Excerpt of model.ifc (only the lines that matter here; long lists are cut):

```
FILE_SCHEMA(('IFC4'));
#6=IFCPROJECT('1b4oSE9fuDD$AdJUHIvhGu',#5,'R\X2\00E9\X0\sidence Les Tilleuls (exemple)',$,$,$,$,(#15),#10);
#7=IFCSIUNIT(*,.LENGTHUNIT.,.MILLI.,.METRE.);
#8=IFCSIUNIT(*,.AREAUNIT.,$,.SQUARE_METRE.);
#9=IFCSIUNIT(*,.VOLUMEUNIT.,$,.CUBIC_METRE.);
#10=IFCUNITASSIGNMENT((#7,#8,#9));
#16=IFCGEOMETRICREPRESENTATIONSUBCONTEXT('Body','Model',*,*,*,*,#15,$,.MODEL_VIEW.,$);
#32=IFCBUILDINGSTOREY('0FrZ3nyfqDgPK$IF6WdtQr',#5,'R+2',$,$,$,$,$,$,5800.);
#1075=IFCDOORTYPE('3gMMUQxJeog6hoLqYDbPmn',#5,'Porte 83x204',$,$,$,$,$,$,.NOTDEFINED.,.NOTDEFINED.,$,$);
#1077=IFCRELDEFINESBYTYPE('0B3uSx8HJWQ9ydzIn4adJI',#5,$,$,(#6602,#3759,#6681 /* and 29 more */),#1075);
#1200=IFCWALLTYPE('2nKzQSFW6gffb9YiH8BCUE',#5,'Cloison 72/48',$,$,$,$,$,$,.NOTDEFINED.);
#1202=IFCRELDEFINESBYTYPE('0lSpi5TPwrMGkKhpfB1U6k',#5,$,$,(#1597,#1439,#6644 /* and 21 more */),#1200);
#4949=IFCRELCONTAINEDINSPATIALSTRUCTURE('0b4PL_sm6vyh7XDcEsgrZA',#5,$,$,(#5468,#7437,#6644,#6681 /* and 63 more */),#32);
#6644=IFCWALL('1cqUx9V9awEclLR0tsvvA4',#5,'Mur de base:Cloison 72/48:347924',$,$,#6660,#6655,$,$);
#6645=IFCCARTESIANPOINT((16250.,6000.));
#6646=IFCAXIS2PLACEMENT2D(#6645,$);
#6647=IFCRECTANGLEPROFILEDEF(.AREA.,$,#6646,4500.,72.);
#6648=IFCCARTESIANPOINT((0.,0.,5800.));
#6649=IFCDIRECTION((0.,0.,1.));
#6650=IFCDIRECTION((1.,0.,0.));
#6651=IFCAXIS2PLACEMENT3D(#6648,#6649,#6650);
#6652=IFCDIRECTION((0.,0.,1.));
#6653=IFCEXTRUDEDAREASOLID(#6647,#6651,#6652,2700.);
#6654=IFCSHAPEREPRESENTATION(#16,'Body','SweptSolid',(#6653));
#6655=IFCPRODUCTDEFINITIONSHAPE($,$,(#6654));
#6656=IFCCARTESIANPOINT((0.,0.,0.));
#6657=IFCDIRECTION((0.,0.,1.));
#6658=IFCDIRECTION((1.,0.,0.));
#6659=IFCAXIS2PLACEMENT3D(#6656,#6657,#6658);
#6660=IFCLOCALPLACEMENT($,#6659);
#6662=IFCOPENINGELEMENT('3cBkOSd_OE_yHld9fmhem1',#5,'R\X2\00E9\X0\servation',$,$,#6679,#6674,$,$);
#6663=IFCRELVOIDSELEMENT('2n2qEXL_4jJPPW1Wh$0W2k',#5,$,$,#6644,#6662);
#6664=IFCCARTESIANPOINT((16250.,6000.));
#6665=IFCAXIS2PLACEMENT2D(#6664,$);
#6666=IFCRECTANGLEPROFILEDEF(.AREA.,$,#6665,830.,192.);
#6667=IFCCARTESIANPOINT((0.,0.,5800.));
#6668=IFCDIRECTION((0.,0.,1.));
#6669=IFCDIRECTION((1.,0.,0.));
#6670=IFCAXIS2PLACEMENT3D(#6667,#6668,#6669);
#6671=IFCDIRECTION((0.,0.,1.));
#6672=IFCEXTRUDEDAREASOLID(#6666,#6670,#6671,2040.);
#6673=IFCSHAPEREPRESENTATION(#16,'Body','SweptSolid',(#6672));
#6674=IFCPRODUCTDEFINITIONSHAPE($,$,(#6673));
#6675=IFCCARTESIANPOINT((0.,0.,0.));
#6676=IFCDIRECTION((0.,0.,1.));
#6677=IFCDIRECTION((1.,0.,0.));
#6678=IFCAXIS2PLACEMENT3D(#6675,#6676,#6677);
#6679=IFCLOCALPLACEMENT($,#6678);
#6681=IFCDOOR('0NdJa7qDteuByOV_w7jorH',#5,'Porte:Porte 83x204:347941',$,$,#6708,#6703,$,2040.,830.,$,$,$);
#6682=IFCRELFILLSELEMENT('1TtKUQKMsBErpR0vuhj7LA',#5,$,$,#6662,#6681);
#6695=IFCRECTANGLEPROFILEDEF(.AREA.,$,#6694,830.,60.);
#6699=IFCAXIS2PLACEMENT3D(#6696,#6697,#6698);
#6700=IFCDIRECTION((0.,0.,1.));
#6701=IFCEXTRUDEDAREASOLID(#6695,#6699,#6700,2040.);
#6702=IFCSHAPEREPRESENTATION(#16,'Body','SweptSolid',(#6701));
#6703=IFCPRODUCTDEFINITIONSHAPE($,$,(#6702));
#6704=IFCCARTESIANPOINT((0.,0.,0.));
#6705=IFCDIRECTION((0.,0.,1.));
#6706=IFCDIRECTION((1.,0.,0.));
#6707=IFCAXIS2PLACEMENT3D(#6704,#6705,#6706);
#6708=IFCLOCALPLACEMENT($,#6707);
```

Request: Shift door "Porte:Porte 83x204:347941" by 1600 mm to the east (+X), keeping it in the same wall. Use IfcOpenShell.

```python
import ifcopenshell
import ifcopenshell.api.geometry
import ifcopenshell.util.placement

model = ifcopenshell.open("model.ifc")

door = model.by_guid("0NdJa7qDteuByOV_w7jorH")
opening = door.FillsVoids[0].RelatingOpeningElement
wall = opening.VoidsElements[0].RelatingBuildingElement

wall_matrix = ifcopenshell.util.placement.get_local_placement(wall.ObjectPlacement)
shift = wall_matrix[:3, 0] * 1600.0
before = ifcopenshell.util.placement.get_local_placement(door.ObjectPlacement)[:3, 3].copy()

# The door is not placed relative to its opening, so move both.
for product in (opening, door):
    matrix = ifcopenshell.util.placement.get_local_placement(product.ObjectPlacement)
    matrix[:3, 3] += shift
    ifcopenshell.api.geometry.edit_object_placement(model, product=product, matrix=matrix, is_si=False)

after = ifcopenshell.util.placement.get_local_placement(door.ObjectPlacement)[:3, 3]
print("door moved by", (after - before).round(3) + 0.0)

model.write("model_edited.ifc")
```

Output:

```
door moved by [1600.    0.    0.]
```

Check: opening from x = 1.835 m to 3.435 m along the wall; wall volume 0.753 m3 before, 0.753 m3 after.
